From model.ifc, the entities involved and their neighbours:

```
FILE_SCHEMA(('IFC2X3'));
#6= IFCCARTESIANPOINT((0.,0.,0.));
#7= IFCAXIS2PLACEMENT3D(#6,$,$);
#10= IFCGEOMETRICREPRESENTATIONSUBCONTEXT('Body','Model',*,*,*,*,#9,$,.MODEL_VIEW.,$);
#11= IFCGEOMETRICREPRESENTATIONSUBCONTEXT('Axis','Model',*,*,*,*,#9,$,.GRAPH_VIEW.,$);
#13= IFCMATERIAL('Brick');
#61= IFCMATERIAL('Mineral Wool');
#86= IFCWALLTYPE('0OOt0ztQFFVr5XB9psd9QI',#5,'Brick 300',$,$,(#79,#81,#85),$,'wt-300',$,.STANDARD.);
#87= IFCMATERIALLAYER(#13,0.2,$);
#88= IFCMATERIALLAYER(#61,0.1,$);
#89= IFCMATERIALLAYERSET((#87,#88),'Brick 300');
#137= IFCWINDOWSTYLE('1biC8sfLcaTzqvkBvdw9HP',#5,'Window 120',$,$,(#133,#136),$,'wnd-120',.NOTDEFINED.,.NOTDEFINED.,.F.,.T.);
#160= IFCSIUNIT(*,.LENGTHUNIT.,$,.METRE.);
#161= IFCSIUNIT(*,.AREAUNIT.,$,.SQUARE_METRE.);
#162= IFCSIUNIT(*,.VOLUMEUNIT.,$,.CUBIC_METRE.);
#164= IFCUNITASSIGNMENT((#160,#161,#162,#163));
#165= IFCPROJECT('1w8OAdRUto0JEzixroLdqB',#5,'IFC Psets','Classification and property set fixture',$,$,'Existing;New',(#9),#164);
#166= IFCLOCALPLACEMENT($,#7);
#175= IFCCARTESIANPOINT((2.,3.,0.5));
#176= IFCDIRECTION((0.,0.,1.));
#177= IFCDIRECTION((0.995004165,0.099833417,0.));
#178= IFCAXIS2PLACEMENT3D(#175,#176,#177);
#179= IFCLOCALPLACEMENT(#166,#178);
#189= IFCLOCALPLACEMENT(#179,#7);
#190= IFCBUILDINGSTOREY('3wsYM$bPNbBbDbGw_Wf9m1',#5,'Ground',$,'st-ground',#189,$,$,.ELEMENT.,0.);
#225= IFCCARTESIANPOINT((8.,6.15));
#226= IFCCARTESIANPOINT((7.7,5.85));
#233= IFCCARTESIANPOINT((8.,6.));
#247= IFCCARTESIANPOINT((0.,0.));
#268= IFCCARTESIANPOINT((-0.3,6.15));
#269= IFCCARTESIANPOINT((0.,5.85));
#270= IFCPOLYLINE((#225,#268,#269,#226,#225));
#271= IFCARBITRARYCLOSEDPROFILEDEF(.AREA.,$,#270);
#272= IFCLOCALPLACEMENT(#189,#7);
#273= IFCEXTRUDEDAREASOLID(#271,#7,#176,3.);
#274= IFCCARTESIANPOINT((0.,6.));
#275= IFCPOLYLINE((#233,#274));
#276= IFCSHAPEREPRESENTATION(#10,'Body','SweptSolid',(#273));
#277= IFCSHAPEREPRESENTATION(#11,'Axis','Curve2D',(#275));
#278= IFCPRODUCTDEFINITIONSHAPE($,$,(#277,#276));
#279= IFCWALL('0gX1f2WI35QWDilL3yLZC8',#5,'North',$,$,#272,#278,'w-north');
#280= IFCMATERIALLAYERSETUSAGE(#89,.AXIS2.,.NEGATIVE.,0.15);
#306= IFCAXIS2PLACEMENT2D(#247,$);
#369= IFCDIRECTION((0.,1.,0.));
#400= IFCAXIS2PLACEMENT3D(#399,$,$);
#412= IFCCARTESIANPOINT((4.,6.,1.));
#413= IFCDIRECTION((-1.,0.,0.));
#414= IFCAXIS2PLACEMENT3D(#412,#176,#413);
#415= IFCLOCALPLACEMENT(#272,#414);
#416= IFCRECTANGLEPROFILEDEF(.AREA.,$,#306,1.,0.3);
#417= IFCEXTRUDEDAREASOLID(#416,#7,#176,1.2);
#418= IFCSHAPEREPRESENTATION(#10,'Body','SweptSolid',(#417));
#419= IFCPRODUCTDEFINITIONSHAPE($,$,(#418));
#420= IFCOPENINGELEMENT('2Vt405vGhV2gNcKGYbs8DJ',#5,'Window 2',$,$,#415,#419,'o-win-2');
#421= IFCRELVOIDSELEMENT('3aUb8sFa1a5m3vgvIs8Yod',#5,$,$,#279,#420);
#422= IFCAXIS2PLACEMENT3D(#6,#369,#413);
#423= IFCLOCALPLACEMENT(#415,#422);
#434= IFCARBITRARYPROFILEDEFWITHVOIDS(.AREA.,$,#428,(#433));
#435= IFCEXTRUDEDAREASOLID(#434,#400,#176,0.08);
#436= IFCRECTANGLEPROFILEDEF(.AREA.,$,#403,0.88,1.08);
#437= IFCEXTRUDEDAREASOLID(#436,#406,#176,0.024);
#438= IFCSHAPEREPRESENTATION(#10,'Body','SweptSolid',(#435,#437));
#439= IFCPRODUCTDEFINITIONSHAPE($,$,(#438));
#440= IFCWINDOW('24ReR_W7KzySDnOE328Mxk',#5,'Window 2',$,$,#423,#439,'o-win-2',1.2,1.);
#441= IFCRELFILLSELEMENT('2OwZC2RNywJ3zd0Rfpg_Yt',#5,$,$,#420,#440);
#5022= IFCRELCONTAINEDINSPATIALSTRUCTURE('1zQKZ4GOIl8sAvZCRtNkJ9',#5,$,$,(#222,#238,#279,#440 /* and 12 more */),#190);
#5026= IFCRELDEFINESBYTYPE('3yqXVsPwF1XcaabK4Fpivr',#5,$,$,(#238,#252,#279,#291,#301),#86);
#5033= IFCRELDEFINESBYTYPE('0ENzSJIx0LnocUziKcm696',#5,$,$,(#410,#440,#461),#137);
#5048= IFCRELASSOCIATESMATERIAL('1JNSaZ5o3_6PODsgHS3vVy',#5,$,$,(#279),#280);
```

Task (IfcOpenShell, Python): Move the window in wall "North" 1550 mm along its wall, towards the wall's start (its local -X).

```python
import ifcopenshell
import ifcopenshell.api.geometry
import ifcopenshell.util.placement

model = ifcopenshell.open("model.ifc")

window = model.by_guid("24ReR_W7KzySDnOE328Mxk")
opening = window.FillsVoids[0].RelatingOpeningElement
wall = opening.VoidsElements[0].RelatingBuildingElement

wall_matrix = ifcopenshell.util.placement.get_local_placement(wall.ObjectPlacement)
shift = wall_matrix[:3, 0] * -1.55
before = ifcopenshell.util.placement.get_local_placement(window.ObjectPlacement)[:3, 3].copy()

# The window is placed relative to its opening, so it follows when the opening moves.
matrix = ifcopenshell.util.placement.get_local_placement(opening.ObjectPlacement)
matrix[:3, 3] += shift
ifcopenshell.api.geometry.edit_object_placement(
    model, product=opening, matrix=matrix, is_si=False, should_transform_children=True
)

after = ifcopenshell.util.placement.get_local_placement(window.ObjectPlacement)[:3, 3]
print("window moved by", (after - before).round(3) + 0.0)

model.write("model_edited.ifc")
```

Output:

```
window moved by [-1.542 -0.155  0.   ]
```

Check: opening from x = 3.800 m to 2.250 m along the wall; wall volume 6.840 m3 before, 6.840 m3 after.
